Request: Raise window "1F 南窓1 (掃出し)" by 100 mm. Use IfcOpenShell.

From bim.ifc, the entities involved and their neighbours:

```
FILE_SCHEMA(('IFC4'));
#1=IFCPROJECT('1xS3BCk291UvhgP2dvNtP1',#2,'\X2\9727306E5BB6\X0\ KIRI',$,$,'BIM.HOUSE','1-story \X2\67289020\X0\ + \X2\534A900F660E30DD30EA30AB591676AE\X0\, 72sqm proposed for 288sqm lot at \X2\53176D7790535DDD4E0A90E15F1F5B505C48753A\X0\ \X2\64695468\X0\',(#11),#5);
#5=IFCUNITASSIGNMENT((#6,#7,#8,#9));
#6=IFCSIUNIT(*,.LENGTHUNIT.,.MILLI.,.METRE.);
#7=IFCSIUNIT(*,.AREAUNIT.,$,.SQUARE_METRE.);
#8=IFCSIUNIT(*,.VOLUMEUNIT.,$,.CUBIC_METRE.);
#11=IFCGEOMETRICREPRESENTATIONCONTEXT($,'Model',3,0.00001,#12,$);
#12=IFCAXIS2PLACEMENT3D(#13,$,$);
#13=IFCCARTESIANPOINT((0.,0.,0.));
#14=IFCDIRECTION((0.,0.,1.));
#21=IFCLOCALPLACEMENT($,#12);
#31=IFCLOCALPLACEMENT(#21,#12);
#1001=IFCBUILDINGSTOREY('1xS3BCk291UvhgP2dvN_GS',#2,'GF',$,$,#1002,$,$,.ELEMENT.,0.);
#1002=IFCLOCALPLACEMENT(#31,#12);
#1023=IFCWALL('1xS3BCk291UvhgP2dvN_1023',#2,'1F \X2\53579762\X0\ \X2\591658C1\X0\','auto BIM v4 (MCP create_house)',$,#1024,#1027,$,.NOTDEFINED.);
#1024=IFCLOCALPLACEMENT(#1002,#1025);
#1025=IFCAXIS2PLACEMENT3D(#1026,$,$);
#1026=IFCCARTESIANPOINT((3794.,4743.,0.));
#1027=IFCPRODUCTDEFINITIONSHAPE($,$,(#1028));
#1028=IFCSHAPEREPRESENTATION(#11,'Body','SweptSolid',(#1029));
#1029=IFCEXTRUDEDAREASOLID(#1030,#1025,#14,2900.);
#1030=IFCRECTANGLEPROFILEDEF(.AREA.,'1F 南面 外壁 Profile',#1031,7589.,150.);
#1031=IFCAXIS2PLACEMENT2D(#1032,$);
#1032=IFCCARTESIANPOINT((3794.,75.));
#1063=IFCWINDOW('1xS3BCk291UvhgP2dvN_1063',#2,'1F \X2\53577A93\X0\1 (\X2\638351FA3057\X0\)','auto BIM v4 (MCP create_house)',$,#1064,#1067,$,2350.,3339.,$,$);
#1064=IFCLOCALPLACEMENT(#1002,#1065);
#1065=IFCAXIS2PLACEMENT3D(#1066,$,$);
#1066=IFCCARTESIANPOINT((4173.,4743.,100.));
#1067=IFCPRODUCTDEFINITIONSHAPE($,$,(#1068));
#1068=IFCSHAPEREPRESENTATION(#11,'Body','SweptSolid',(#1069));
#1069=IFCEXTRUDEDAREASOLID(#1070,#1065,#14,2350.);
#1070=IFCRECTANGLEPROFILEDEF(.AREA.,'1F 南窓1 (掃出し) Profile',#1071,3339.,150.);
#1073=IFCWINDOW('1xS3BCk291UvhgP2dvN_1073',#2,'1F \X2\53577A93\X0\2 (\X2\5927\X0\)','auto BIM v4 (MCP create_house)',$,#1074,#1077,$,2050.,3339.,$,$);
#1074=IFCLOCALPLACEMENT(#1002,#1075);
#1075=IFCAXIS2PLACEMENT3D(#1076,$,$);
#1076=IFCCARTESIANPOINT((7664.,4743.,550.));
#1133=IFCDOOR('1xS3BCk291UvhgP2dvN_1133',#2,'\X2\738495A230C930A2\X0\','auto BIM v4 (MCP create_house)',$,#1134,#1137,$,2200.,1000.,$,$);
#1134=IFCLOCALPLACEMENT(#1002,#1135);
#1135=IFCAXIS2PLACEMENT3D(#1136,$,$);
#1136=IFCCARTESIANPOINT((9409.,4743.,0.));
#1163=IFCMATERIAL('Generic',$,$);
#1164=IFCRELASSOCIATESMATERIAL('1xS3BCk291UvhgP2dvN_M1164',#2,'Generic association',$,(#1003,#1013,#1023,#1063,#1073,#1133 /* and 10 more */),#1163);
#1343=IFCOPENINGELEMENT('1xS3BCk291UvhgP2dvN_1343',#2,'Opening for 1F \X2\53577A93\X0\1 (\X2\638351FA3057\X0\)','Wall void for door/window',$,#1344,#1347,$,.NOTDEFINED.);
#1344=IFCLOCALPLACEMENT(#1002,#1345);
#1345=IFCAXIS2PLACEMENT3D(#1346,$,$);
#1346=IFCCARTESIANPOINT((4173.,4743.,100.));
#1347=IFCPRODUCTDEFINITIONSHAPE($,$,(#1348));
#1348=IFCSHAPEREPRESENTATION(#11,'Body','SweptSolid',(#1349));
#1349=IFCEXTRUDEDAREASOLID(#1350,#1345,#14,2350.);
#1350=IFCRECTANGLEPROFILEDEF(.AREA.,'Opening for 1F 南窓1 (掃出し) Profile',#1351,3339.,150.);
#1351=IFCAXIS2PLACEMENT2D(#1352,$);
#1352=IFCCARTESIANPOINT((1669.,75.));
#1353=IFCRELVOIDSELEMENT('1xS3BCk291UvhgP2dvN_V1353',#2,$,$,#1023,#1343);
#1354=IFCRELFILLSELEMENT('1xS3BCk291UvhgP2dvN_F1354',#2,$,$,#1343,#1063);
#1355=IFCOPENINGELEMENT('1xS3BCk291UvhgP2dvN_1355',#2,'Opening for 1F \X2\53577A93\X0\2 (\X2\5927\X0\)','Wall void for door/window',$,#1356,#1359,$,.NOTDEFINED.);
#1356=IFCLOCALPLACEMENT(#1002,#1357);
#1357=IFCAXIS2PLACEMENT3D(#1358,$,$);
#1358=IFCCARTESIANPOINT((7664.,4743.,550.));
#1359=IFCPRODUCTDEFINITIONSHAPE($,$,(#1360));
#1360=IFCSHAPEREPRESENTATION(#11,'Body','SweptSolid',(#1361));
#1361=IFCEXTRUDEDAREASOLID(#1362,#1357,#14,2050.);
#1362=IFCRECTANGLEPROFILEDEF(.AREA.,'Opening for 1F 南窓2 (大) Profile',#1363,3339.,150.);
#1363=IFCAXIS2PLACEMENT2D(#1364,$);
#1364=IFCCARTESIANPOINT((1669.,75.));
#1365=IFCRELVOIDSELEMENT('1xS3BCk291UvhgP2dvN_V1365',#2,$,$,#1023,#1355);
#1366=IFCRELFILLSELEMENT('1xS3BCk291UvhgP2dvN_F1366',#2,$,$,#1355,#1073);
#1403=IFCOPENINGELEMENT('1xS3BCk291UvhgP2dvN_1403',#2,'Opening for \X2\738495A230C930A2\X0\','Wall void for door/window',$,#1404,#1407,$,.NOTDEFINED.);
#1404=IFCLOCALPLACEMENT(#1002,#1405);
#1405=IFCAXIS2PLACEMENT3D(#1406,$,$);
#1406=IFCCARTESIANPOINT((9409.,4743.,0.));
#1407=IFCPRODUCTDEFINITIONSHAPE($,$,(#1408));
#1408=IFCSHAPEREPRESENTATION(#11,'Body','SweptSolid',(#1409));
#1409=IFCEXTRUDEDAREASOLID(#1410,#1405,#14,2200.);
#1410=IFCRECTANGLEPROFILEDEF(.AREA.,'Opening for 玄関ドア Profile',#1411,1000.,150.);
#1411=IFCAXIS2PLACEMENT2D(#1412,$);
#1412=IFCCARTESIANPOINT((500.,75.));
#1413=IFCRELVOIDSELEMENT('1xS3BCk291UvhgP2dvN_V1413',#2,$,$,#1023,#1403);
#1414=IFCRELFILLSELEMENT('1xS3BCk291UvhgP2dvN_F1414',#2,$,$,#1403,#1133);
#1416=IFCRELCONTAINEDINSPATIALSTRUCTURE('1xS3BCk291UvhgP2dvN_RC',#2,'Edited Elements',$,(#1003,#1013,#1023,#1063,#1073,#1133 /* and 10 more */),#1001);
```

```python
import numpy as np
import ifcopenshell
import ifcopenshell.api.geometry
import ifcopenshell.util.placement
import ifcopenshell.util.unit

model = ifcopenshell.open("bim.ifc")
unit_scale = ifcopenshell.util.unit.calculate_unit_scale(model)

window = model.by_guid("1xS3BCk291UvhgP2dvN_1063")
opening = window.FillsVoids[0].RelatingOpeningElement
dz = 100.0

shift = np.array([0.0, 0.0, dz])
# The window is not placed relative to its opening, so move both.
for product in (opening, window):
    matrix = ifcopenshell.util.placement.get_local_placement(product.ObjectPlacement)
    matrix[:3, 3] += shift
    ifcopenshell.api.geometry.edit_object_placement(model, product=product, matrix=matrix, is_si=False)

print(f"moved by {dz * unit_scale:+.3f} m")

model.write("bim_updated.ifc")
```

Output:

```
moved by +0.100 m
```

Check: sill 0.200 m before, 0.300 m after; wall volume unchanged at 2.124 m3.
